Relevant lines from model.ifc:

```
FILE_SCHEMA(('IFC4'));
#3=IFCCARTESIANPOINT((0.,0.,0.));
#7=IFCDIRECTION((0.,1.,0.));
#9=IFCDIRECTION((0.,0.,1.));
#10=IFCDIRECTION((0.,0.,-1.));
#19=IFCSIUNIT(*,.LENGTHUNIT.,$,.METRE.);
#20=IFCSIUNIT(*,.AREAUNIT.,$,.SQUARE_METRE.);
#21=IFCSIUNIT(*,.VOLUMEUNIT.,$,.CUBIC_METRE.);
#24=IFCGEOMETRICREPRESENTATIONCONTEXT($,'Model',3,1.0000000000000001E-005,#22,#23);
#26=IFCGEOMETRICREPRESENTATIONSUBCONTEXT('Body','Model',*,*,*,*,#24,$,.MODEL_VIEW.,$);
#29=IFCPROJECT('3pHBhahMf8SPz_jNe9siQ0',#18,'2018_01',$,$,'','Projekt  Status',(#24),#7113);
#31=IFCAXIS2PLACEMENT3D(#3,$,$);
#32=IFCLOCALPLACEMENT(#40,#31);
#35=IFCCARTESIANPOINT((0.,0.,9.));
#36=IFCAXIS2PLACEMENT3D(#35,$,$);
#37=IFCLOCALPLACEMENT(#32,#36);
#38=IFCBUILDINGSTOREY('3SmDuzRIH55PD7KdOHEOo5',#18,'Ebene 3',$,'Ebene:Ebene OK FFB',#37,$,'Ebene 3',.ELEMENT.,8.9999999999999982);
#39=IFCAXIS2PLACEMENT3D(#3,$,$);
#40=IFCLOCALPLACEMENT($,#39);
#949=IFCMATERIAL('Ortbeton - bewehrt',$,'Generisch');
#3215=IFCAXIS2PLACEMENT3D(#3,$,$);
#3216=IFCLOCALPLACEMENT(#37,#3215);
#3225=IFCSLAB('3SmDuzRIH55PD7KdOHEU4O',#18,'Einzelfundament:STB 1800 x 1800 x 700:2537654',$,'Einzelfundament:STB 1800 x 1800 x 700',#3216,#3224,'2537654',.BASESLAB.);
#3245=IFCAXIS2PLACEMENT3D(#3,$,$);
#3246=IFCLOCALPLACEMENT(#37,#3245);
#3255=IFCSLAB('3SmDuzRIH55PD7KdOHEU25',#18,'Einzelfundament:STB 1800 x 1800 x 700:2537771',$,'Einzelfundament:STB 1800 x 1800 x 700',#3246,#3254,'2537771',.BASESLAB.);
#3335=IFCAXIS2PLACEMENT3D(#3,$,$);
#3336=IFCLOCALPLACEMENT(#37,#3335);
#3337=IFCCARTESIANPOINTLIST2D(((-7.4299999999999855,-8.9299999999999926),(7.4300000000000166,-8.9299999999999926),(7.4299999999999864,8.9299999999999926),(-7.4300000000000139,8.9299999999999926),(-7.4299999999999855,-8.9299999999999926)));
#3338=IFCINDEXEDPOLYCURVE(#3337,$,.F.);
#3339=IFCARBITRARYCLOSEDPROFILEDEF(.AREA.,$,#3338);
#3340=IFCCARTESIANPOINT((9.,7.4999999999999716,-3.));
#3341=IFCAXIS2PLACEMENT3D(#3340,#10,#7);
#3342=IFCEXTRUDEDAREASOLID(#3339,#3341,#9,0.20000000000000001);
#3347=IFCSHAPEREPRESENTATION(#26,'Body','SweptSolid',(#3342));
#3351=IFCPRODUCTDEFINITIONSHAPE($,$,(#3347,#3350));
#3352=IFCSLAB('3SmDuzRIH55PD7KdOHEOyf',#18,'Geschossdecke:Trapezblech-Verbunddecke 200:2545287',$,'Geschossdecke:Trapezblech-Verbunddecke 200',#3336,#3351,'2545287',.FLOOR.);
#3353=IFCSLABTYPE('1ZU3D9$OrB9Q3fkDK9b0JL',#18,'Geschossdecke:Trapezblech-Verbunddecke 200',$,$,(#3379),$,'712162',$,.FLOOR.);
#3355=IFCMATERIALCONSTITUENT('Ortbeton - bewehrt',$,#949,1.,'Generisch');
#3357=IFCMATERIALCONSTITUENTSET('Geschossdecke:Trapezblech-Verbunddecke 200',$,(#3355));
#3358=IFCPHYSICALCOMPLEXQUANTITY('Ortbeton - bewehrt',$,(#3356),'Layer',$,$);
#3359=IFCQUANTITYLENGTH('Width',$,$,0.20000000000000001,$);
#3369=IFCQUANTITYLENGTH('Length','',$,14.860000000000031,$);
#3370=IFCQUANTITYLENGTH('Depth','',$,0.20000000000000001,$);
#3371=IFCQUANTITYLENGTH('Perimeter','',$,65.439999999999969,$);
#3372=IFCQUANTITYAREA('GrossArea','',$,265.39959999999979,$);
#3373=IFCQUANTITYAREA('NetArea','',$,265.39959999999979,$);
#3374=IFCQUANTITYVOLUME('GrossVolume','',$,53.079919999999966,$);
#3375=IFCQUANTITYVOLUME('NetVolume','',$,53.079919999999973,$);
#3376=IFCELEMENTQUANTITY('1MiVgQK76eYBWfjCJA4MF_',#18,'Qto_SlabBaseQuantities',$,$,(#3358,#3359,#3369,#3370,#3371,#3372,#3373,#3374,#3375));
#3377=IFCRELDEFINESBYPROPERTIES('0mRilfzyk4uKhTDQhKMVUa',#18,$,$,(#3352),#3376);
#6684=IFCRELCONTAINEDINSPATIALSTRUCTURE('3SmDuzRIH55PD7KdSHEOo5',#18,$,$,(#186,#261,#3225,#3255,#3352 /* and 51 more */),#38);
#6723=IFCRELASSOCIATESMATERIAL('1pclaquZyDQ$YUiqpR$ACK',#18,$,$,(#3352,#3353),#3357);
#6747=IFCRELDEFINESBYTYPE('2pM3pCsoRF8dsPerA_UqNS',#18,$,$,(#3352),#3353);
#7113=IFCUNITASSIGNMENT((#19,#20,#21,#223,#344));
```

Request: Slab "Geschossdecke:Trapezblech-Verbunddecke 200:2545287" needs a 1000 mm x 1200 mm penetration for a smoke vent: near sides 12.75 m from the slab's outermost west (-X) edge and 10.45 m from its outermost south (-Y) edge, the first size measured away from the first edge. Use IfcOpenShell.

```python
import numpy as np
import ifcopenshell
import ifcopenshell.api.feature
import ifcopenshell.api.geometry
import ifcopenshell.api.pset
import ifcopenshell.api.root
import ifcopenshell.geom
import ifcopenshell.util.element
import ifcopenshell.util.placement
import ifcopenshell.util.representation
import ifcopenshell.util.shape
import ifcopenshell.util.unit

model = ifcopenshell.open("model.ifc")
unit_scale = ifcopenshell.util.unit.calculate_unit_scale(model)
area_scale = ifcopenshell.util.unit.calculate_unit_scale(model, "AREAUNIT")
volume_scale = ifcopenshell.util.unit.calculate_unit_scale(model, "VOLUMEUNIT")
settings = ifcopenshell.geom.settings()


def volume(element):
    """Net volume in cubic metres, openings subtracted."""
    shape = ifcopenshell.geom.create_shape(settings, element)
    return ifcopenshell.util.shape.get_volume(shape.geometry)


slab = model.by_guid("3SmDuzRIH55PD7KdOHEOyf")
before = volume(slab)

# Extent in the slab's own axes, in metres. The edges named are its -X and -Y sides.
slab_shape = ifcopenshell.geom.create_shape(settings, slab)
vertices = ifcopenshell.util.shape.get_vertices(slab_shape.geometry)
x_min, y_min, bottom = vertices.min(axis=0)
top = vertices[:, 2].max()

opening = ifcopenshell.api.root.create_entity(model, ifc_class="IfcOpeningElement", name="Smoke vent opening", predefined_type="OPENING")
context = ifcopenshell.util.representation.get_context(model, "Model", "Body", "MODEL_VIEW")
width, depth = 1, 1.2
outline = [(0.0, 0.0), (width, 0.0), (width, depth), (0.0, depth), (0.0, 0.0)]
# Overshoot both faces by 50 mm so the cut is clean.
shape = ifcopenshell.api.geometry.add_slab_representation(
    model, context=context, depth=top - bottom + 0.1, polyline=outline
)
ifcopenshell.api.geometry.assign_representation(model, product=opening, representation=shape)

matrix = ifcopenshell.util.placement.get_local_placement(slab.ObjectPlacement)
matrix[:, 3] = matrix @ np.append(np.array([x_min + 12.75, y_min + 10.45, bottom - 0.05]) / unit_scale, 1.0)
ifcopenshell.api.geometry.edit_object_placement(model, product=opening, matrix=matrix, is_si=False)
ifcopenshell.api.feature.add_feature(model, feature=opening, element=slab)

after = volume(slab)

# Update the slab's stored quantities.
qto = model.by_id(ifcopenshell.util.element.get_pset(slab, "Qto_SlabBaseQuantities", should_inherit=False)["id"])
ifcopenshell.api.pset.edit_qto(model, qto=qto, properties={
    "NetArea": after / (top - bottom) / area_scale,
    "NetVolume": after / volume_scale,
})

print(f"slab volume {before:.3f} -> {after:.3f} m3")

model.write("model_updated.ifc")
```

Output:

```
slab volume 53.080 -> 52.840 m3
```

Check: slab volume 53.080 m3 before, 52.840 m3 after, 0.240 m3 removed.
